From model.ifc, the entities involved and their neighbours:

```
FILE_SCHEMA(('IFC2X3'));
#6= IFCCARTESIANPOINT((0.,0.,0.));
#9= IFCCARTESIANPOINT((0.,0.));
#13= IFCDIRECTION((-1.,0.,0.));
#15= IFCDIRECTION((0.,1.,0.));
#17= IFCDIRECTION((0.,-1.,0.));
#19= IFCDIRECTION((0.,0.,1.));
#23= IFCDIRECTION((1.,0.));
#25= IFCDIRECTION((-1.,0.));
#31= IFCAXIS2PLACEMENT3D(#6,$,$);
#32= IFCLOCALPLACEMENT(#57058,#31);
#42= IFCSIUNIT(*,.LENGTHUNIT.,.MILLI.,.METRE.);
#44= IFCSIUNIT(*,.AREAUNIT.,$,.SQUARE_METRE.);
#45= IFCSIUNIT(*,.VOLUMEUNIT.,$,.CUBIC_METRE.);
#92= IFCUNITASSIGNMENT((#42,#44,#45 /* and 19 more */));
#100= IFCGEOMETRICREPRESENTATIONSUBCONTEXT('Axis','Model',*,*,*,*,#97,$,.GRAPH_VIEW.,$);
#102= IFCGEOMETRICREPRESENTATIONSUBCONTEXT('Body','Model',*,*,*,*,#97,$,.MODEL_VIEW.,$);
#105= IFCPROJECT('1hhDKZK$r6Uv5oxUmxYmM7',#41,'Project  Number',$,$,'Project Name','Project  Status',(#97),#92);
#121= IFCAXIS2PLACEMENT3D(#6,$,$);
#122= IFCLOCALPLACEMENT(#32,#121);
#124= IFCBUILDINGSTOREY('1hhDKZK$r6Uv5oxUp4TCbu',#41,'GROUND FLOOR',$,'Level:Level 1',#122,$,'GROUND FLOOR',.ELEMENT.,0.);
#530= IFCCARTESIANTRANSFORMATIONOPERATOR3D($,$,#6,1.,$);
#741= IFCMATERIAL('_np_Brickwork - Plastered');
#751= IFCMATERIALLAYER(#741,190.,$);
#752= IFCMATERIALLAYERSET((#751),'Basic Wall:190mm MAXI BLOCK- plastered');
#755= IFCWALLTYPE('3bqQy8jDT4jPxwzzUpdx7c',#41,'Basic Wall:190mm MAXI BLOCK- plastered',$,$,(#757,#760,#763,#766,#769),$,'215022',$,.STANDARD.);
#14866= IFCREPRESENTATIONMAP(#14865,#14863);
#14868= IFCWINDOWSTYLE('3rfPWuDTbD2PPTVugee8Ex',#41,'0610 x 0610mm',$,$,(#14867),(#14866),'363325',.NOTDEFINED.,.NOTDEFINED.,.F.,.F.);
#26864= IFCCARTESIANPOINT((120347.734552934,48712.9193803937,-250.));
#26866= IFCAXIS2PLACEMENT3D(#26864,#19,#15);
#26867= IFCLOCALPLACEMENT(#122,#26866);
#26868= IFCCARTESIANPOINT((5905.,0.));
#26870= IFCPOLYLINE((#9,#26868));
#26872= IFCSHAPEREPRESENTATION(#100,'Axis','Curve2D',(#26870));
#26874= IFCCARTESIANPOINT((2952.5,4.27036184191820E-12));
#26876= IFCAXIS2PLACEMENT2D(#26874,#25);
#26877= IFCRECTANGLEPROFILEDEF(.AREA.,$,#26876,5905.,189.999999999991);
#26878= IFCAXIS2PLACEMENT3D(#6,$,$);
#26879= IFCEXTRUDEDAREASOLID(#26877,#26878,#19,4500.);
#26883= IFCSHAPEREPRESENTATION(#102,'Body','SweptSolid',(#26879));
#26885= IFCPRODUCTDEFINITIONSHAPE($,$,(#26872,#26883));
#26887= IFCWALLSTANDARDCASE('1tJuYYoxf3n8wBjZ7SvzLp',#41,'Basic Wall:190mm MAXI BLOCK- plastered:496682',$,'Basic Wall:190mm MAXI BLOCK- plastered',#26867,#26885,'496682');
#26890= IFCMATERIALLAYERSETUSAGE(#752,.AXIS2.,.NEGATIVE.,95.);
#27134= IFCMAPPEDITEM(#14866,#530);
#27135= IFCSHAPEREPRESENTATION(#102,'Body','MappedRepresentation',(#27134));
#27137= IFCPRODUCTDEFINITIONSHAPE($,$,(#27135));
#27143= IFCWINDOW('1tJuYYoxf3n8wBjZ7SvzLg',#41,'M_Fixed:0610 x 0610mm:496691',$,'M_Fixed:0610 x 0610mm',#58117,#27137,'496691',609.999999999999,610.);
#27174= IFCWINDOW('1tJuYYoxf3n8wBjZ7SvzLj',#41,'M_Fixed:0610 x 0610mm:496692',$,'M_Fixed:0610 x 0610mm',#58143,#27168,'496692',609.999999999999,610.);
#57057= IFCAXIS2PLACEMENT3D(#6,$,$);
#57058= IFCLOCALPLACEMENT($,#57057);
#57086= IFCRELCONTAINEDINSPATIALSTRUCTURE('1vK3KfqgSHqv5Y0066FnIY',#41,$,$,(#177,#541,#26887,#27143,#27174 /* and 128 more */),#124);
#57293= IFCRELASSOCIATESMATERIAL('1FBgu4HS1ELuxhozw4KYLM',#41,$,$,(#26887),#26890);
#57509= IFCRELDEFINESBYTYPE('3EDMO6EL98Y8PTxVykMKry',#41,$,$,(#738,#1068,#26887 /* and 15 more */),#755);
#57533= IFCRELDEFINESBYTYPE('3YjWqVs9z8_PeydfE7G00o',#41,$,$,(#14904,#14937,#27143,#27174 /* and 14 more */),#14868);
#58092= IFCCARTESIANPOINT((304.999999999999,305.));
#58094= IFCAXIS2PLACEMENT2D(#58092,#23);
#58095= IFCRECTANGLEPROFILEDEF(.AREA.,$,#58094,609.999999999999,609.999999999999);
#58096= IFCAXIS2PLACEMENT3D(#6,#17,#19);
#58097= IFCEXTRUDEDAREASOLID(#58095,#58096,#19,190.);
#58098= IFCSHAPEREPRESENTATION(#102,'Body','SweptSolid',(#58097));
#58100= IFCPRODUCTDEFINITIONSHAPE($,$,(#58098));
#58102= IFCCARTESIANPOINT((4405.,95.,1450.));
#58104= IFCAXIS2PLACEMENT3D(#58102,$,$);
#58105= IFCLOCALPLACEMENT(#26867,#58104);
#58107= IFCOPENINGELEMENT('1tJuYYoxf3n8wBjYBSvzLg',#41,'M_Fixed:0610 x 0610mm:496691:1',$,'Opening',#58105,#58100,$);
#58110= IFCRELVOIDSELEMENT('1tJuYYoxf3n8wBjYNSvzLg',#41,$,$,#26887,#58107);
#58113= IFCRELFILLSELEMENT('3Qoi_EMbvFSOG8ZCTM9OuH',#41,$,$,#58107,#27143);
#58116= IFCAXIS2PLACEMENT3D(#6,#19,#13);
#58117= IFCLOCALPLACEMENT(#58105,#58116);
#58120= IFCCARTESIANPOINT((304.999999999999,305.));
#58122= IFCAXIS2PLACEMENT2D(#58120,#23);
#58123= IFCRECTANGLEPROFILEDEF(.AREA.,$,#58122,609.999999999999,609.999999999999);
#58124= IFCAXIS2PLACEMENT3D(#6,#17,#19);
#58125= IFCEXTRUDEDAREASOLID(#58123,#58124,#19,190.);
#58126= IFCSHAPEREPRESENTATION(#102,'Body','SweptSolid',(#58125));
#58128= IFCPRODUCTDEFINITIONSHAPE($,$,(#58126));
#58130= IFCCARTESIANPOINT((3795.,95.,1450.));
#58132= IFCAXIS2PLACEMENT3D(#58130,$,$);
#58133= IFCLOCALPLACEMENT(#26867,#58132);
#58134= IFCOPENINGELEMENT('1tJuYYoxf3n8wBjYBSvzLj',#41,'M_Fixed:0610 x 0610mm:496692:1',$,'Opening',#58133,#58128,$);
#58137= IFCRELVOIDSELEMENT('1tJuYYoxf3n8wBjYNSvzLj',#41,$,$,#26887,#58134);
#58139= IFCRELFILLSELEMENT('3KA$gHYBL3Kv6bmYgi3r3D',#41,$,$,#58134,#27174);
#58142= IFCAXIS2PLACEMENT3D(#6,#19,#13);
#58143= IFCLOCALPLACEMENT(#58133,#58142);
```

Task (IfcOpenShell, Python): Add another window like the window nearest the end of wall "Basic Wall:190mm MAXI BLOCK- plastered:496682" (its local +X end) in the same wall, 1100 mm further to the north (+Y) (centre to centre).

```python
import ifcopenshell
import ifcopenshell.api.feature
import ifcopenshell.api.geometry
import ifcopenshell.api.root
import ifcopenshell.geom
import ifcopenshell.util.element
import ifcopenshell.util.placement
import ifcopenshell.util.shape

model = ifcopenshell.open("model.ifc")
settings = ifcopenshell.geom.settings()


def volume(element):
    """Net volume in cubic metres, openings subtracted."""
    shape = ifcopenshell.geom.create_shape(settings, element)
    return ifcopenshell.util.shape.get_volume(shape.geometry)


def reuse_history(source, copy):
    """copy_class also copies each property set's owner history, people and application; keep the originals."""
    for rel in copy.IsDefinedBy:
        if rel.is_a("IfcRelDefinesByProperties") and (history := rel.RelatingPropertyDefinition.OwnerHistory):
            rel.RelatingPropertyDefinition.OwnerHistory = source.OwnerHistory
            ifcopenshell.util.element.remove_deep2(model, history)


window = model.by_id(27143)
opening = window.FillsVoids[0].RelatingOpeningElement
wall = opening.VoidsElements[0].RelatingBuildingElement
before = volume(wall)
shift = ifcopenshell.util.placement.get_local_placement(wall.ObjectPlacement)[:3, 0] * 1100.0

# copy_class copies the void relationship, type, container and properties, but no geometry.
new_opening = ifcopenshell.api.root.copy_class(model, product=opening)
new_opening.Representation = ifcopenshell.util.element.copy_deep(
    model, opening.Representation, exclude=["IfcGeometricRepresentationContext", "IfcRepresentationMap"]
)
new_opening.Name = "M_Fixed:0610 x 0610mm"
new_window = ifcopenshell.api.root.copy_class(model, product=window)
new_window.Representation = ifcopenshell.util.element.copy_deep(
    model, window.Representation, exclude=["IfcGeometricRepresentationContext", "IfcRepresentationMap"]
)
new_window.Name = "M_Fixed:0610 x 0610mm"
new_window.Tag = None
reuse_history(window, new_window)
fills = ifcopenshell.api.feature.add_filling(model, opening=new_opening, element=new_window)
fills.OwnerHistory = new_window.OwnerHistory  # required in IFC2X3

for old, new in ((opening, new_opening), (window, new_window)):
    matrix = ifcopenshell.util.placement.get_local_placement(old.ObjectPlacement)
    matrix[:3, 3] += shift
    ifcopenshell.api.geometry.edit_object_placement(model, product=new, matrix=matrix, is_si=False)

after = volume(wall)

print(f"wall volume {before:.3f} -> {after:.3f} m3")

model.write("model_edited.ifc")
```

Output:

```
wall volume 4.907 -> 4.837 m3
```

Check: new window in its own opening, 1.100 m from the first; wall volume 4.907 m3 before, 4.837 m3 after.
